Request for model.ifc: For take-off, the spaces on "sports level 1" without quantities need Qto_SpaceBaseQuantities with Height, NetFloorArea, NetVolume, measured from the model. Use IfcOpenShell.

First a look at what the model holds.

```python
import ifcopenshell
import ifcopenshell.util.element
import ifcopenshell.util.unit

model = ifcopenshell.open("model.ifc")
print(model.schema)
for unit_type in ("LENGTHUNIT", "AREAUNIT", "VOLUMEUNIT"):
    print(unit_type, ifcopenshell.util.unit.calculate_unit_scale(model, unit_type))
storey = next(s for s in model.by_type("IfcBuildingStorey") if s.Name == "sports level 1")
spaces = [e for e in ifcopenshell.util.element.get_decomposition(storey) if e.is_a("IfcSpace")]
for e in sorted(spaces, key=lambda e: e.id()):
    print(e.id(), e.is_a(), e.Name, list(ifcopenshell.util.element.get_psets(e, qtos_only=True)), sep=" | ")
```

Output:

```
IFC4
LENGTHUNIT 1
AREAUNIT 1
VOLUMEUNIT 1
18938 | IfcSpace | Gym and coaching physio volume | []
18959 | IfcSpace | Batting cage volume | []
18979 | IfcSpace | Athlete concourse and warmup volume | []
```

```python
import ifcopenshell
import ifcopenshell.api.pset
import ifcopenshell.geom
import ifcopenshell.util.element
import ifcopenshell.util.shape
import ifcopenshell.util.unit

model = ifcopenshell.open("model.ifc")
unit_scale = ifcopenshell.util.unit.calculate_unit_scale(model)
area_scale = ifcopenshell.util.unit.calculate_unit_scale(model, "AREAUNIT")
volume_scale = ifcopenshell.util.unit.calculate_unit_scale(model, "VOLUMEUNIT")
settings = ifcopenshell.geom.settings()

storey = next(s for s in model.by_type("IfcBuildingStorey") if s.Name == "sports level 1")
spaces = [e for e in ifcopenshell.util.element.get_decomposition(storey) if e.is_a("IfcSpace")]

for e in sorted(spaces, key=lambda e: e.id()):
    if ifcopenshell.util.element.get_psets(e, qtos_only=True, should_inherit=False):
        continue
    # Geometry comes back in metres, in the element's own axes.
    shape = ifcopenshell.geom.create_shape(settings, e)
    values = {
        "Height": ifcopenshell.util.shape.get_z(shape.geometry) / unit_scale,
        "NetFloorArea": ifcopenshell.util.shape.get_footprint_area(shape.geometry) / area_scale,
        "NetVolume": ifcopenshell.util.shape.get_volume(shape.geometry) / volume_scale,
    }
    qto = ifcopenshell.api.pset.add_qto(model, product=e, name="Qto_SpaceBaseQuantities")
    ifcopenshell.api.pset.edit_qto(model, qto=qto, properties=values)
    print(e.id(), {k: round(v, 3) for k, v in values.items()})

model.write("model_rev.ifc")
```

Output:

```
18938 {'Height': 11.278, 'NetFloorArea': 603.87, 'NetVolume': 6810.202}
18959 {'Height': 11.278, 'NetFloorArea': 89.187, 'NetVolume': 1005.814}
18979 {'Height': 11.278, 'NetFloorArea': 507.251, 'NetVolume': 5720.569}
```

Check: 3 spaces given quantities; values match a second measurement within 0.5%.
